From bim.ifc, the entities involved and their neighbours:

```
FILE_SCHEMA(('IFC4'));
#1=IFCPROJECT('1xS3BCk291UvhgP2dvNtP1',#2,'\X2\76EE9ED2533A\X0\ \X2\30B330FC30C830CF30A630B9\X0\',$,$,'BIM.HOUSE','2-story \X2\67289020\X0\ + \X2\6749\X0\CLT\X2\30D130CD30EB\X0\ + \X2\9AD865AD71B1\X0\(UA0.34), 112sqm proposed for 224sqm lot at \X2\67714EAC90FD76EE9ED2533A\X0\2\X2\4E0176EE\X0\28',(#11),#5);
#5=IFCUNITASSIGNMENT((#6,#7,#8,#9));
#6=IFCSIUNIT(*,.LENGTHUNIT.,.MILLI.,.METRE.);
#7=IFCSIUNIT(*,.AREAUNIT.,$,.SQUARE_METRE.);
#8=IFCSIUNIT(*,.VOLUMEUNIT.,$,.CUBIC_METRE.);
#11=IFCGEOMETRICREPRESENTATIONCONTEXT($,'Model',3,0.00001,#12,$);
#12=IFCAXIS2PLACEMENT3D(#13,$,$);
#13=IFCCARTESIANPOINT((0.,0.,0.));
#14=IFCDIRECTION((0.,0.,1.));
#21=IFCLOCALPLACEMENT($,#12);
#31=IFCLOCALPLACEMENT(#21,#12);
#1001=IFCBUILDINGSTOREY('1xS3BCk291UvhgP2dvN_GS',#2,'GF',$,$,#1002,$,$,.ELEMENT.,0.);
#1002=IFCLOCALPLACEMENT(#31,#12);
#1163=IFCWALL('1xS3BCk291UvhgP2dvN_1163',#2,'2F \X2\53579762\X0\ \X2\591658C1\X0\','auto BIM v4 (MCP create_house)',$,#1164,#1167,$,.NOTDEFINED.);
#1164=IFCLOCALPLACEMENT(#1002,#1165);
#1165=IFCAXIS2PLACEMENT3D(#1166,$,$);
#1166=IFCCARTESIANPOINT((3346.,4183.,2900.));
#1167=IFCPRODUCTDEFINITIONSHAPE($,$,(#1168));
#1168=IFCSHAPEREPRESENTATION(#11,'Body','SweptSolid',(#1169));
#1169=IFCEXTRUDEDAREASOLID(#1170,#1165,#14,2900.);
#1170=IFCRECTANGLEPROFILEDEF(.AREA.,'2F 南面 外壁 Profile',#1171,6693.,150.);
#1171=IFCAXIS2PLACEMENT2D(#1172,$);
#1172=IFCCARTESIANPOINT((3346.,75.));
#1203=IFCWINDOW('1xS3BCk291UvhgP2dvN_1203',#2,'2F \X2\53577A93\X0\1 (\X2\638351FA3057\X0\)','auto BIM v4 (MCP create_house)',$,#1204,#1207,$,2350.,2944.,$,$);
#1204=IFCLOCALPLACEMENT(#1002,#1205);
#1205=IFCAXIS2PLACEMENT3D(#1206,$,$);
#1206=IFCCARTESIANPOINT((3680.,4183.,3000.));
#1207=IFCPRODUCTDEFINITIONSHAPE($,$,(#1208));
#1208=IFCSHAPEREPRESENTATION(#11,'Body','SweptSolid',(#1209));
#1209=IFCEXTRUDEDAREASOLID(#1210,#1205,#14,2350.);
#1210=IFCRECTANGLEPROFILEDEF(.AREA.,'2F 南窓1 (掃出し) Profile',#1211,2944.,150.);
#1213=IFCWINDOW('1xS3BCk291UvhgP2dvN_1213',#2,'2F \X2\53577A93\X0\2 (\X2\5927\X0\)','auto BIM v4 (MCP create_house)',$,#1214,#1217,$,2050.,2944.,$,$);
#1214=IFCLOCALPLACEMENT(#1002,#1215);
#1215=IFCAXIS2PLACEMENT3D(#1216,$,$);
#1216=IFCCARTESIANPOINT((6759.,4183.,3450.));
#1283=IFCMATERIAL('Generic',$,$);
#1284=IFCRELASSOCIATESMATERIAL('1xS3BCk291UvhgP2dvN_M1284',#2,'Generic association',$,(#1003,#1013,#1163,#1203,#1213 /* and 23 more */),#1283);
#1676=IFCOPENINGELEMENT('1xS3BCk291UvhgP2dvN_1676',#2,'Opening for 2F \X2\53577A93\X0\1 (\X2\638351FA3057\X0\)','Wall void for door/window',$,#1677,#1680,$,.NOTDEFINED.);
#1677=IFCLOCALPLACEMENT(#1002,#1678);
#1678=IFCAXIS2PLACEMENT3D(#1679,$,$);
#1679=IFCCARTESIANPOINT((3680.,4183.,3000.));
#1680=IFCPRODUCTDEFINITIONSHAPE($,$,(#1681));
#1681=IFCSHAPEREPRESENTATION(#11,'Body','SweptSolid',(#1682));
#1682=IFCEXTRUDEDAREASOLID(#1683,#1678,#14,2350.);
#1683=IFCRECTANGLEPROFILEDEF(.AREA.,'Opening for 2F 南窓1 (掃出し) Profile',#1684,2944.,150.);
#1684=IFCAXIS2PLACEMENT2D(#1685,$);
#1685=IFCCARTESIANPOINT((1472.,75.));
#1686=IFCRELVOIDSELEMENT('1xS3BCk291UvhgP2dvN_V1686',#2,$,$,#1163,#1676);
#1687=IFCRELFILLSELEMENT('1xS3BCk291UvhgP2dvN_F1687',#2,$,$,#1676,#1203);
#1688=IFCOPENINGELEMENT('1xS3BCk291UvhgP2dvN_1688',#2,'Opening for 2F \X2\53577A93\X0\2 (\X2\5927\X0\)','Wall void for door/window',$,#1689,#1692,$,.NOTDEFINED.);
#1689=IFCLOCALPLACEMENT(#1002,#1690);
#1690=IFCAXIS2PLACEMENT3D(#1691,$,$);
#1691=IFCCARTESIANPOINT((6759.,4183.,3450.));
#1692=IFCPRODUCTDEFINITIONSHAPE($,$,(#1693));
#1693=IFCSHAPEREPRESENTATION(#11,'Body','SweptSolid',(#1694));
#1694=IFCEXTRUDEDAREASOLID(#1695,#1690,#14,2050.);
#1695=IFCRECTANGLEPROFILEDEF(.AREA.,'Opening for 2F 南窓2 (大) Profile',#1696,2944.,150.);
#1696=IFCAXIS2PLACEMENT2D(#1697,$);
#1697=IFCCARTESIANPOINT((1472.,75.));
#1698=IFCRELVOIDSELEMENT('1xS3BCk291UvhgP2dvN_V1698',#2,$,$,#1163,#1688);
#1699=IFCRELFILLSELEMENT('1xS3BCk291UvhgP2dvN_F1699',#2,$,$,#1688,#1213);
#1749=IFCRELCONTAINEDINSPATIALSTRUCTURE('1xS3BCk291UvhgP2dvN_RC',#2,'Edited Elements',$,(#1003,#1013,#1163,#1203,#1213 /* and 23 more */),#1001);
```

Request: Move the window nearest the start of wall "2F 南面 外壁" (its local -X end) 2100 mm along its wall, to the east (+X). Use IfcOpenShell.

```python
import ifcopenshell
import ifcopenshell.api.geometry
import ifcopenshell.util.placement
import ifcopenshell.util.unit

model = ifcopenshell.open("bim.ifc")
unit_scale = ifcopenshell.util.unit.calculate_unit_scale(model)

window = model.by_id(1203)
opening = window.FillsVoids[0].RelatingOpeningElement
wall = opening.VoidsElements[0].RelatingBuildingElement

wall_matrix = ifcopenshell.util.placement.get_local_placement(wall.ObjectPlacement)
shift = wall_matrix[:3, 0] * 2.1 / unit_scale
before = ifcopenshell.util.placement.get_local_placement(window.ObjectPlacement)[:3, 3].copy()

# The window is not placed relative to its opening, so move both.
for product in (opening, window):
    matrix = ifcopenshell.util.placement.get_local_placement(product.ObjectPlacement)
    matrix[:3, 3] += shift
    ifcopenshell.api.geometry.edit_object_placement(model, product=product, matrix=matrix, is_si=False)

after = ifcopenshell.util.placement.get_local_placement(window.ObjectPlacement)[:3, 3]
print("window moved by", (after - before).round(3) + 0.0)

model.write("bim_updated.ifc")
```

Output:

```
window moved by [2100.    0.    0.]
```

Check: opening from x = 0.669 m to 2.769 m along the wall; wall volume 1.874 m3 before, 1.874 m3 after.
